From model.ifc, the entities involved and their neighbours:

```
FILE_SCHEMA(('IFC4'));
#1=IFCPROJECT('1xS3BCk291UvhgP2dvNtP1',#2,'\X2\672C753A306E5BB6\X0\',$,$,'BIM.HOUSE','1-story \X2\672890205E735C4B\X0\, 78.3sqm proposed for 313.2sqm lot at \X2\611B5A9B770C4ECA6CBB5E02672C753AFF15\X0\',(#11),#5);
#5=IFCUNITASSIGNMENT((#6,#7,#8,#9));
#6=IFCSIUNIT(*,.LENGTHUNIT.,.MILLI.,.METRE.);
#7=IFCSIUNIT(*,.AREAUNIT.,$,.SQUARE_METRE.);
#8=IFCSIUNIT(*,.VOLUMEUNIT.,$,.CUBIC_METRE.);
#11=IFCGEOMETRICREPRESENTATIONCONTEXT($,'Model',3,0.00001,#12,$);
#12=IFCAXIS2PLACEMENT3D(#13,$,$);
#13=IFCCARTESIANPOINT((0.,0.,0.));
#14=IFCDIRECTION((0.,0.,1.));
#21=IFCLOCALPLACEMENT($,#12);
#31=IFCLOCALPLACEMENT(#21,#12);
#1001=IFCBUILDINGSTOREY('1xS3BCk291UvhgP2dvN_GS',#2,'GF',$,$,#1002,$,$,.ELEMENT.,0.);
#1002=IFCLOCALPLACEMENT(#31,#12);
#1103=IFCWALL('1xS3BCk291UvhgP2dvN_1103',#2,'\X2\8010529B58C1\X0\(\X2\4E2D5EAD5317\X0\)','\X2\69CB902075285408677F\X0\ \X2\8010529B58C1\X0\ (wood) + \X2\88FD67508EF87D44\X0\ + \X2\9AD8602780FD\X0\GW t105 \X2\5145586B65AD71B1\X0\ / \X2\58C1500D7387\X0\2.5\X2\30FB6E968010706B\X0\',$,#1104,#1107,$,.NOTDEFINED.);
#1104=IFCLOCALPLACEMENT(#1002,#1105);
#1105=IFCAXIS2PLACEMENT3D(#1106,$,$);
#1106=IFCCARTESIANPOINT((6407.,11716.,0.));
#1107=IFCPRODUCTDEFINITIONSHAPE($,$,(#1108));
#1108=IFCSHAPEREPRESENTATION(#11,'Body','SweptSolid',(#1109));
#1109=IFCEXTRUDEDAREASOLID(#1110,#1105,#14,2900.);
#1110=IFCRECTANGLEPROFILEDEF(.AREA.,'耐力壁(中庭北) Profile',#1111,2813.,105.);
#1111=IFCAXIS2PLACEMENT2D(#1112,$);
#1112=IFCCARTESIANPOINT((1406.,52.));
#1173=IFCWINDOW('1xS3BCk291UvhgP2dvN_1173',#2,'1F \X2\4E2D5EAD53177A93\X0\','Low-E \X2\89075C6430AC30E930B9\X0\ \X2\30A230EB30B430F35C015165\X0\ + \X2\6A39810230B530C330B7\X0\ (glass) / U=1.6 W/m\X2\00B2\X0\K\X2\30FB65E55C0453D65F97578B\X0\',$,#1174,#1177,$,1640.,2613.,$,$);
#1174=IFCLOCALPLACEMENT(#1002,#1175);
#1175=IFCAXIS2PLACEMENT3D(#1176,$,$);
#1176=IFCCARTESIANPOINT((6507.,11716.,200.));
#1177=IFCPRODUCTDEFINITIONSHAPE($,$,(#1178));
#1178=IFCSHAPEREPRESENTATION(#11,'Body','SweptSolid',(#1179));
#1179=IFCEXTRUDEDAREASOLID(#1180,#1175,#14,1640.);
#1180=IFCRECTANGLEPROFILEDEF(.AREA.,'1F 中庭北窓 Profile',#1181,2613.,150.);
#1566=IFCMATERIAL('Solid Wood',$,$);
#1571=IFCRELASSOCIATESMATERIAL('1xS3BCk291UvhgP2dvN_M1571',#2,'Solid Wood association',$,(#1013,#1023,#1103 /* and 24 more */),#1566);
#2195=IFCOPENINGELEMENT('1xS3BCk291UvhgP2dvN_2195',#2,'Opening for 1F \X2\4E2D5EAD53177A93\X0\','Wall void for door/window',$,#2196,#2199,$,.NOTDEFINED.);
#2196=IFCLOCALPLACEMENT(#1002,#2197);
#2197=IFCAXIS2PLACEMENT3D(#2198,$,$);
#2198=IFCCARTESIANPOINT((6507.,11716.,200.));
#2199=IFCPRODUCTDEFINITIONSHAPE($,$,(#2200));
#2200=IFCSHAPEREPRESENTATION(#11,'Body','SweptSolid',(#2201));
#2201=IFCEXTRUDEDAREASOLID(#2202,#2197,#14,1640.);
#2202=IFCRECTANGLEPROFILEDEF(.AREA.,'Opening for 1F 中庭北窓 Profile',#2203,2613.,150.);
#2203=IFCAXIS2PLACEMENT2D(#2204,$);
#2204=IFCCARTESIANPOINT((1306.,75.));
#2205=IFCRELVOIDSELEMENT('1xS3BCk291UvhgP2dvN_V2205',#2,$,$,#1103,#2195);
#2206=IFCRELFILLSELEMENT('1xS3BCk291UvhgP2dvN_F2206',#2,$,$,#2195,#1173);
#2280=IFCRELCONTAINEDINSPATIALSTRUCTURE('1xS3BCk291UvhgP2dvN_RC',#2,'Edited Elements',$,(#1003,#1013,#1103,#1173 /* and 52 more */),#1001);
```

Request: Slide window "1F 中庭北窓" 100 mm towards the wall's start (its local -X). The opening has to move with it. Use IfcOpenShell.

```python
import ifcopenshell
import ifcopenshell.api.geometry
import ifcopenshell.util.placement
import ifcopenshell.util.unit

model = ifcopenshell.open("model.ifc")
unit_scale = ifcopenshell.util.unit.calculate_unit_scale(model)

window = model.by_guid("1xS3BCk291UvhgP2dvN_1173")
opening = window.FillsVoids[0].RelatingOpeningElement
wall = opening.VoidsElements[0].RelatingBuildingElement

wall_matrix = ifcopenshell.util.placement.get_local_placement(wall.ObjectPlacement)
shift = wall_matrix[:3, 0] * -0.1 / unit_scale
before = ifcopenshell.util.placement.get_local_placement(window.ObjectPlacement)[:3, 3].copy()

# The window is not placed relative to its opening, so move both.
for product in (opening, window):
    matrix = ifcopenshell.util.placement.get_local_placement(product.ObjectPlacement)
    matrix[:3, 3] += shift
    ifcopenshell.api.geometry.edit_object_placement(model, product=product, matrix=matrix, is_si=False)

after = ifcopenshell.util.placement.get_local_placement(window.ObjectPlacement)[:3, 3]
print("window moved by", (after - before).round(3) + 0.0)

model.write("model_updated.ifc")
```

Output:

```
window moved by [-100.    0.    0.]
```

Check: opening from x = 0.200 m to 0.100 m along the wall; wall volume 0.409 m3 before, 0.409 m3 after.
